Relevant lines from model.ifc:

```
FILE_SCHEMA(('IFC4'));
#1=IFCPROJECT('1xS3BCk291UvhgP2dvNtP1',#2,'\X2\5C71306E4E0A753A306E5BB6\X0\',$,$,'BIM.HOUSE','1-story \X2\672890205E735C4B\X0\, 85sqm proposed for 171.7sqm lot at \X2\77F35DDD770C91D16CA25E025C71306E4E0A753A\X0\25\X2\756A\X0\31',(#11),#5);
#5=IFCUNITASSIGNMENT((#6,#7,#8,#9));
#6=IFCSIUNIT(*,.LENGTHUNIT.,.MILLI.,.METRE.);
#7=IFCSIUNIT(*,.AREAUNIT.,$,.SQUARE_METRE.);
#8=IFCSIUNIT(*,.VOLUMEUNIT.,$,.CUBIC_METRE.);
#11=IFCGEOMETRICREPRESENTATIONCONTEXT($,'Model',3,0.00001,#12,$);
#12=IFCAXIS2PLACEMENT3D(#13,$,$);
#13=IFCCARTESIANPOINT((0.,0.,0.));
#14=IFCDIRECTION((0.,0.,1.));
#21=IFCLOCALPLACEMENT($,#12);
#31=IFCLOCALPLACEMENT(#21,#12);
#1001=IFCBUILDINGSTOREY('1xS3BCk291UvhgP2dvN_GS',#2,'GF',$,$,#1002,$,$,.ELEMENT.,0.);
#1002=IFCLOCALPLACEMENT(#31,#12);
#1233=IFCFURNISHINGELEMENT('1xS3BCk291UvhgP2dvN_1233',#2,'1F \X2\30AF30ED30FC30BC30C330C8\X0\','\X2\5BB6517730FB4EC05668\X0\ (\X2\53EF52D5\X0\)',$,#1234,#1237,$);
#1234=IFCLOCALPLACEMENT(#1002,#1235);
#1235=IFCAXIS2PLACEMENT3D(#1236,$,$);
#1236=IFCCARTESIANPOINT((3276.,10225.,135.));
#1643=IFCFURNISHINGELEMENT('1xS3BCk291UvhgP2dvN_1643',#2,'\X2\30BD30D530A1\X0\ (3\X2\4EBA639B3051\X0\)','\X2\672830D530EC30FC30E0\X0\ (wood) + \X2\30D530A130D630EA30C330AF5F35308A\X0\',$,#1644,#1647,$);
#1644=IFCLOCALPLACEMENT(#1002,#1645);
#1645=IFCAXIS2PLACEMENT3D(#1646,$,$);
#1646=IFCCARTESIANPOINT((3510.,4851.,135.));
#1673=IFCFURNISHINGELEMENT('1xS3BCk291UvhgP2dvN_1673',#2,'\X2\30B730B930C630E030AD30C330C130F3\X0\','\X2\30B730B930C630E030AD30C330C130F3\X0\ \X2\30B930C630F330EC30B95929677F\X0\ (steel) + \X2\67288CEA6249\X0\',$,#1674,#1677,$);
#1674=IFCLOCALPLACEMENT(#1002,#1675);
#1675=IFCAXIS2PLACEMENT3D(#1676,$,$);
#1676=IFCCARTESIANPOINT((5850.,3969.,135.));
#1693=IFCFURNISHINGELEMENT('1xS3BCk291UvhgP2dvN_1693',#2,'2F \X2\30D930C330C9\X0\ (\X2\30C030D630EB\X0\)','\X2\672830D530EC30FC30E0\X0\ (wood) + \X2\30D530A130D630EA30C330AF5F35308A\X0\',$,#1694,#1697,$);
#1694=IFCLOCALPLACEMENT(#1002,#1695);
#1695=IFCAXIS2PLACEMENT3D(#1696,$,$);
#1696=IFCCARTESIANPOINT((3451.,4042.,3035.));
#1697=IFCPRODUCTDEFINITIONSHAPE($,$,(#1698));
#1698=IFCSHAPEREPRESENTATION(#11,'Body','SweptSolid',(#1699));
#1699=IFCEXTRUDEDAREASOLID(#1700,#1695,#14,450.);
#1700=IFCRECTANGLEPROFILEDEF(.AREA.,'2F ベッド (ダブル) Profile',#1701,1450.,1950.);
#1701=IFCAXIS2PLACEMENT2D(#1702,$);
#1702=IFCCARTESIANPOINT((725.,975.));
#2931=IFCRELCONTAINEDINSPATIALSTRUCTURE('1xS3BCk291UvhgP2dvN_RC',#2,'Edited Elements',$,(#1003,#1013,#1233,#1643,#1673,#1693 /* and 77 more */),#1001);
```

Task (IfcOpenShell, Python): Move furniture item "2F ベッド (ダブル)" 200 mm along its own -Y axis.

```python
import ifcopenshell
import ifcopenshell.api.geometry
import ifcopenshell.util.placement

model = ifcopenshell.open("model.ifc")

item = model.by_guid("1xS3BCk291UvhgP2dvN_1693")
matrix = ifcopenshell.util.placement.get_local_placement(item.ObjectPlacement)
matrix[:3, 3] -= matrix[:3, 1] * 200.0
ifcopenshell.api.geometry.edit_object_placement(model, product=item, matrix=matrix, is_si=False)

print(ifcopenshell.util.placement.get_local_placement(item.ObjectPlacement).round(3) + 0.0)

model.write("model_edited.ifc")
```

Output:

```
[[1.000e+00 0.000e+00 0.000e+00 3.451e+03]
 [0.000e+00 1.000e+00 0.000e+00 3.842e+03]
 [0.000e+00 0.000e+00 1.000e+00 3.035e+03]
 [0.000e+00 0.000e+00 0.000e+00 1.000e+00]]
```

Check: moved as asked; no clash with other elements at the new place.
